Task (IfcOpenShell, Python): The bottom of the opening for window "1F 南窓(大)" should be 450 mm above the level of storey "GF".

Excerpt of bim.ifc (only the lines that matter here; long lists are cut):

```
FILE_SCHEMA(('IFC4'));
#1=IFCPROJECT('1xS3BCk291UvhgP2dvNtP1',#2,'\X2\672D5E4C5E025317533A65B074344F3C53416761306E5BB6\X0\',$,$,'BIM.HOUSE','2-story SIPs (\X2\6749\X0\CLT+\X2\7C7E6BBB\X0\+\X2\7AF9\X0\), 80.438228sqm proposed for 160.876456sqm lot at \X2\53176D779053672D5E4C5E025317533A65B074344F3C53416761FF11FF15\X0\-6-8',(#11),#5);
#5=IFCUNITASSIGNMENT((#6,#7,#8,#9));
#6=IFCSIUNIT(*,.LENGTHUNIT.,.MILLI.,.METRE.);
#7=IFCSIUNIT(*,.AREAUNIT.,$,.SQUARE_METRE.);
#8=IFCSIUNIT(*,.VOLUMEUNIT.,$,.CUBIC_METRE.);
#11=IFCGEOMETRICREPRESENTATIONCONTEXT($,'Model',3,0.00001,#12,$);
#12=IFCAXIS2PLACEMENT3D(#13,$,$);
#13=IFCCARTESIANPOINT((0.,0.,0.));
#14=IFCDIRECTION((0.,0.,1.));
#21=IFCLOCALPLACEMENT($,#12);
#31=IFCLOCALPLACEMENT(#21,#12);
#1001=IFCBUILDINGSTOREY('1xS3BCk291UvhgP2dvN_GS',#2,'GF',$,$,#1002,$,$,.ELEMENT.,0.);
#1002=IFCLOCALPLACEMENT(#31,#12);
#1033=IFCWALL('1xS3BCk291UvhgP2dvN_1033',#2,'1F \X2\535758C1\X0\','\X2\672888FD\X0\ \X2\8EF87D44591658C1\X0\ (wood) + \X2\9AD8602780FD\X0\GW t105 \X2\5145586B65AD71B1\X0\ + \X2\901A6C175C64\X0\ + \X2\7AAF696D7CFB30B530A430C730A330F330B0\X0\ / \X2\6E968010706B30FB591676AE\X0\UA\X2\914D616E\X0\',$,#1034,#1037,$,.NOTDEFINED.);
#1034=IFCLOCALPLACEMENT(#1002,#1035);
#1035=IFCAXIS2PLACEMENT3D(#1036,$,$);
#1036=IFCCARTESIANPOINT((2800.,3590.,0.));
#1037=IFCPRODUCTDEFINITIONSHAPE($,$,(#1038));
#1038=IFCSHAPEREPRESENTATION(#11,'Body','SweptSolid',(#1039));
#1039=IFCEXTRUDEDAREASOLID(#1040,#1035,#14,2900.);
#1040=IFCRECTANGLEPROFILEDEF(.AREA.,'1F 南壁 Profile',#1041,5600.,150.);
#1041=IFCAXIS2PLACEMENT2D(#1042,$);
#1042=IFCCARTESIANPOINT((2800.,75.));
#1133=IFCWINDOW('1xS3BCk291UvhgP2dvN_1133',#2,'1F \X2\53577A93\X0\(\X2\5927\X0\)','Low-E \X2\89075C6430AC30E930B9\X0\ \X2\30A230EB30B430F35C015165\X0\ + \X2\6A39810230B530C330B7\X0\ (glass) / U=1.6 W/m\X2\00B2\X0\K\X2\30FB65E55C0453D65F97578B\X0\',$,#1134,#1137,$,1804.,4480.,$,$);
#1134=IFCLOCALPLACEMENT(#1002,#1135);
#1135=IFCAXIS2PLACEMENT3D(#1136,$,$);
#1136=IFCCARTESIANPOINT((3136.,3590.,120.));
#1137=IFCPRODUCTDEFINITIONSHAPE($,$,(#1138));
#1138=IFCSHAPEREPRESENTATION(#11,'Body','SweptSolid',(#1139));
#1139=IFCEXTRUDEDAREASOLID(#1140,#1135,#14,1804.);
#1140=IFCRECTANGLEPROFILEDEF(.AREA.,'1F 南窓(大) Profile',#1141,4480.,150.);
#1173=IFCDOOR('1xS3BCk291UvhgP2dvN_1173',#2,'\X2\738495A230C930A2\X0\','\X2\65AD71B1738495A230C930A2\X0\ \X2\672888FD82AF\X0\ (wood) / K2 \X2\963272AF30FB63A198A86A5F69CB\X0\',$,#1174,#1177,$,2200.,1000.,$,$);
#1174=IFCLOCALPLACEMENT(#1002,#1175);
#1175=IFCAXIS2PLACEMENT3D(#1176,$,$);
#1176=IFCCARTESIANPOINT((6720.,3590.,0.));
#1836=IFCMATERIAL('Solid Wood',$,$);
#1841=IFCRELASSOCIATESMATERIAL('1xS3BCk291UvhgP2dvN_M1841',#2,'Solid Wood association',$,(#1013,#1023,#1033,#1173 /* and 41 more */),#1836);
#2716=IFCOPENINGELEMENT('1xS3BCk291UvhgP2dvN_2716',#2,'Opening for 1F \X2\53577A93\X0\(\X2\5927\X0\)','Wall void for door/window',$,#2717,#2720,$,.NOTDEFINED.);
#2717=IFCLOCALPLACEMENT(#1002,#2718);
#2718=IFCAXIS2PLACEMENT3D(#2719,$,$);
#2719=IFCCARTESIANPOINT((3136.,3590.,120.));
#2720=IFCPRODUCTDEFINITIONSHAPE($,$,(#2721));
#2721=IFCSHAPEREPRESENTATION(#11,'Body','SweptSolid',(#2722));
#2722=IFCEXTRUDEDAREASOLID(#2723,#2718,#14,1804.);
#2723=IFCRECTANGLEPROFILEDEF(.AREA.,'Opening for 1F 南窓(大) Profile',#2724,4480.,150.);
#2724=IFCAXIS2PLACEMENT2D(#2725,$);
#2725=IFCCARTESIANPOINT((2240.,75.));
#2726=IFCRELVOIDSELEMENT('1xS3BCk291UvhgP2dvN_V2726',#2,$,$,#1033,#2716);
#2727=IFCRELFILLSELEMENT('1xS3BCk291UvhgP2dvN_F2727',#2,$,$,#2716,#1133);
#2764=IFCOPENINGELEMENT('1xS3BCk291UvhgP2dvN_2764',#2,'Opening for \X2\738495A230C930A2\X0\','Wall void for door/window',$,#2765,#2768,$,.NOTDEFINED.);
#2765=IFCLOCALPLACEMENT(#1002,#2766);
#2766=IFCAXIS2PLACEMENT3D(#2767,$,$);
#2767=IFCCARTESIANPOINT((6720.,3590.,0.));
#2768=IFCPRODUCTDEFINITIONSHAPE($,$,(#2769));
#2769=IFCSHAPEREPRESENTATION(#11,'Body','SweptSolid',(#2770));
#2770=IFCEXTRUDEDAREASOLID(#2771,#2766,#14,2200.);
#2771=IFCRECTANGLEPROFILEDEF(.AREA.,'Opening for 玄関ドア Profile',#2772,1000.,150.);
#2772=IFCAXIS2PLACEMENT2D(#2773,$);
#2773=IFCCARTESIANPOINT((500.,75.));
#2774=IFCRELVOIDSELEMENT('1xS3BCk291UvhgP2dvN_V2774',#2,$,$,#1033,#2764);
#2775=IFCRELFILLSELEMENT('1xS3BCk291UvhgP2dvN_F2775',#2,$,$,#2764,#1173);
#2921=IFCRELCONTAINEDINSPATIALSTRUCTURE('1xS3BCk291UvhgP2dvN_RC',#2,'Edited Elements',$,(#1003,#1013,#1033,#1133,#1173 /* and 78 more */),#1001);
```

```python
import numpy as np
import ifcopenshell
import ifcopenshell.api.geometry
import ifcopenshell.geom
import ifcopenshell.util.element
import ifcopenshell.util.placement
import ifcopenshell.util.shape
import ifcopenshell.util.unit

model = ifcopenshell.open("bim.ifc")
unit_scale = ifcopenshell.util.unit.calculate_unit_scale(model)

window = model.by_guid("1xS3BCk291UvhgP2dvN_1133")
opening = window.FillsVoids[0].RelatingOpeningElement
storey = ifcopenshell.util.element.get_container(window, ifc_class="IfcBuildingStorey")
level = ifcopenshell.util.placement.get_local_placement(storey.ObjectPlacement)[2, 3]

# The opening's origin need not be at the sill, so measure its lowest point.
shape = ifcopenshell.geom.create_shape(ifcopenshell.geom.settings(), opening)
bottom = ifcopenshell.util.shape.get_shape_bottom_elevation(shape, shape.geometry) / unit_scale
dz = level + 0.45 / unit_scale - bottom

shift = np.array([0.0, 0.0, dz])
# The window is not placed relative to its opening, so move both.
for product in (opening, window):
    matrix = ifcopenshell.util.placement.get_local_placement(product.ObjectPlacement)
    matrix[:3, 3] += shift
    ifcopenshell.api.geometry.edit_object_placement(model, product=product, matrix=matrix, is_si=False)

print(f"moved by {dz * unit_scale:+.3f} m")

model.write("bim_edited.ifc")
```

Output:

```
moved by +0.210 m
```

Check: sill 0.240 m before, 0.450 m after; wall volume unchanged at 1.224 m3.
